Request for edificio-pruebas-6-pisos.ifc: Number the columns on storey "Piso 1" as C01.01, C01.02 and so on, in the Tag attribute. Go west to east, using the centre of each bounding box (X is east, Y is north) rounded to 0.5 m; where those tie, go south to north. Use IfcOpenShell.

First a look at what the model holds.

```python
import ifcopenshell
import ifcopenshell.util.element
import ifcopenshell.util.placement

model = ifcopenshell.open("edificio-pruebas-6-pisos.ifc")
print(model.schema)
storey = next(s for s in model.by_type("IfcBuildingStorey") if s.Name == "Piso 1")
columns = [e for e in ifcopenshell.util.element.get_decomposition(storey) if e.is_a("IfcColumn")]
for e in sorted(columns, key=lambda e: e.id()):
    origin = ifcopenshell.util.placement.get_local_placement(e.ObjectPlacement)[:3, 3]
    print(e.id(), e.Tag, e.Name, origin.round(2) + 0.0, sep=" | ")
```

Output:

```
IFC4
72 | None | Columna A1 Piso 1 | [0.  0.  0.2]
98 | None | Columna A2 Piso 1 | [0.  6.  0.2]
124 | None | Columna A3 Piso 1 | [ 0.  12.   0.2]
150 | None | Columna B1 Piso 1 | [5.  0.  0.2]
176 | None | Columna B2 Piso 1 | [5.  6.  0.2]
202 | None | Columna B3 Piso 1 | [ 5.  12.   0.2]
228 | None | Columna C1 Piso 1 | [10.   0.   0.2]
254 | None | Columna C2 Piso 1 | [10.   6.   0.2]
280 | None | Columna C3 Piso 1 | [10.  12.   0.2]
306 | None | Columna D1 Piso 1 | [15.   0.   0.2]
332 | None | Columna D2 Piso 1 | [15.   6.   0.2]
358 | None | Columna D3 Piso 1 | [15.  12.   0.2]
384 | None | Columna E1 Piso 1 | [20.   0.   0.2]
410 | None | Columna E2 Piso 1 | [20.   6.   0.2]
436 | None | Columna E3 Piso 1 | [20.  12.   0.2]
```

```python
import ifcopenshell
import ifcopenshell.geom
import ifcopenshell.util.element
import ifcopenshell.util.shape

model = ifcopenshell.open("edificio-pruebas-6-pisos.ifc")
settings = ifcopenshell.geom.settings()
settings.set("use-world-coords", True)


def centre(element):
    shape = ifcopenshell.geom.create_shape(settings, element)
    return ifcopenshell.util.shape.get_bbox_centroid(shape.geometry)


storey = next(s for s in model.by_type("IfcBuildingStorey") if s.Name == "Piso 1")
columns = [e for e in ifcopenshell.util.element.get_decomposition(storey) if e.is_a("IfcColumn")]

# Insertion points can sit at a corner or the storey origin, so sort by the geometry (in metres).
centres = {e: centre(e) for e in columns}
columns.sort(key=lambda e: (round(centres[e][0] / 0.5), centres[e][1]))

for i, e in enumerate(columns, start=1):
    number = f"C01.{i:02d}"
    e.Tag = number
    print(e.id(), number)

model.write("edificio-pruebas-6-pisos_v2.ifc")
```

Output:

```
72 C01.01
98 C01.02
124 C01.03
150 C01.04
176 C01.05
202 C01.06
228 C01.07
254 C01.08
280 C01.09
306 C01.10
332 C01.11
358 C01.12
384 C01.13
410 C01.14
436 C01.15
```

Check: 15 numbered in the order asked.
